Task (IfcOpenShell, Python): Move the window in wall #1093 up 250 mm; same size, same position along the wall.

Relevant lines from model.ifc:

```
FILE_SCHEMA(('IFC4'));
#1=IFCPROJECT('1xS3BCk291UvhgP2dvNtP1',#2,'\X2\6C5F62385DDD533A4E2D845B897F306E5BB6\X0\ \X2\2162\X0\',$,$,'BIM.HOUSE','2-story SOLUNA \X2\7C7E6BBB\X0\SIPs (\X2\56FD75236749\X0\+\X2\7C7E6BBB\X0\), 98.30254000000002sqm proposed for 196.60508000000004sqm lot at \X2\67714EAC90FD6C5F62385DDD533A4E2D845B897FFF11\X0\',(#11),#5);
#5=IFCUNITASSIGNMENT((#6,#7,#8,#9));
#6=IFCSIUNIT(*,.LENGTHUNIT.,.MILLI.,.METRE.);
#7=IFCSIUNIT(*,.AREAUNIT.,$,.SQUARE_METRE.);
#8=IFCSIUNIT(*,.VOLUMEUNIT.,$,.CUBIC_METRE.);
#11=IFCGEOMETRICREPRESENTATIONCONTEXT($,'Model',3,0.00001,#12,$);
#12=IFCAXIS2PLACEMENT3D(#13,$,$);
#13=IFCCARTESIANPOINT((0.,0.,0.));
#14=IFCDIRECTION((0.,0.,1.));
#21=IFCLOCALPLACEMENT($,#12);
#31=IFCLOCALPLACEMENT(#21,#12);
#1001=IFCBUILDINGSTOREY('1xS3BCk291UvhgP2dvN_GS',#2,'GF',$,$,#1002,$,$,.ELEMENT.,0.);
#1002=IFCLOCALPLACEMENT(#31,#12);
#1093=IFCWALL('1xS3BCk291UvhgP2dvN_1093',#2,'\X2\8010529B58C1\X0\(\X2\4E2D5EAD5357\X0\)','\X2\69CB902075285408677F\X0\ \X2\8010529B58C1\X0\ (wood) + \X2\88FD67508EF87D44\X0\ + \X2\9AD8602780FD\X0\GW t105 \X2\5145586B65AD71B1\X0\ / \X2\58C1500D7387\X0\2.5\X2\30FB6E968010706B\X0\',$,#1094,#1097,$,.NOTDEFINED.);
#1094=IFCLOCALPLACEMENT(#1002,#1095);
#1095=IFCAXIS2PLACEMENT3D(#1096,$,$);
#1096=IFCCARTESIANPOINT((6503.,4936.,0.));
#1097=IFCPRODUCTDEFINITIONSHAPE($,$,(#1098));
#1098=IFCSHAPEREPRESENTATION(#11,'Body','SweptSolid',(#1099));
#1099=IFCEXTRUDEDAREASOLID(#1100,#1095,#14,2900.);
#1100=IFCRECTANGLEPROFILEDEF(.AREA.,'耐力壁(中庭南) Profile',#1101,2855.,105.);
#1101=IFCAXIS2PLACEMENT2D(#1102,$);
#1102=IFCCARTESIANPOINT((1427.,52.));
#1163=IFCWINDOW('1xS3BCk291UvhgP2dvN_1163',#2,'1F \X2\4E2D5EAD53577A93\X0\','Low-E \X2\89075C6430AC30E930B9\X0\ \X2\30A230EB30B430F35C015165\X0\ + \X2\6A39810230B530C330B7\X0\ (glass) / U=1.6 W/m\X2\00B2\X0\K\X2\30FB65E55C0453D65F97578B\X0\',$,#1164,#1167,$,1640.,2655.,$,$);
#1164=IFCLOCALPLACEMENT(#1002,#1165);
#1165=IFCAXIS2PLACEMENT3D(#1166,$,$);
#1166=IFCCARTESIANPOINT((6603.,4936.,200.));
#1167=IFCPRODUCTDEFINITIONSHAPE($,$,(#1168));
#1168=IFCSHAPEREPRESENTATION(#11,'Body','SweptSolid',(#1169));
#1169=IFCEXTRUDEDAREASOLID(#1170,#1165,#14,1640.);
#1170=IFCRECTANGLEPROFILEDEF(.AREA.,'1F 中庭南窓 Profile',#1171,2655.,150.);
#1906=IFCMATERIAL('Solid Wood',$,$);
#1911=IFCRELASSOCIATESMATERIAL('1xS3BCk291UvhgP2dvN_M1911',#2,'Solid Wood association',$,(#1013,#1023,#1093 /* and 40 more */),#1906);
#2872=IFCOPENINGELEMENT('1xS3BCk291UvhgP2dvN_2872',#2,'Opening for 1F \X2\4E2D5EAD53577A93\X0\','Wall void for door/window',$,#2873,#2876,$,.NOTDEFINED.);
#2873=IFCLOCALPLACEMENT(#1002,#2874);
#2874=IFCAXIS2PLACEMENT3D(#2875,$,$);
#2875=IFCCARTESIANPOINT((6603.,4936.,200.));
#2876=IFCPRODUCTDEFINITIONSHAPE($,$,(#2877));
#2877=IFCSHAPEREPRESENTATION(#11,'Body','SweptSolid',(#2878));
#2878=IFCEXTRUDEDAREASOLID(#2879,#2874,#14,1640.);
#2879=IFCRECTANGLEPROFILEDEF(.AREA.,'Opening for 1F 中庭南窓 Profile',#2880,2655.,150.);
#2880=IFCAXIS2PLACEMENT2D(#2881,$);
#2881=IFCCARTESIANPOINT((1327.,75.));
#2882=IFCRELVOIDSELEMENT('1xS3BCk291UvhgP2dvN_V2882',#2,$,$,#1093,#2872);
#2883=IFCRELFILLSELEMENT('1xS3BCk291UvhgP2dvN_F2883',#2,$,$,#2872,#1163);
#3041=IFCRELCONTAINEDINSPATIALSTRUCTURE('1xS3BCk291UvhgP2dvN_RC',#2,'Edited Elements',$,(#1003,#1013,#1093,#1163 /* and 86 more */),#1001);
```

```python
import numpy as np
import ifcopenshell
import ifcopenshell.api.geometry
import ifcopenshell.util.placement
import ifcopenshell.util.unit

model = ifcopenshell.open("model.ifc")
unit_scale = ifcopenshell.util.unit.calculate_unit_scale(model)

window = model.by_id(1163)
opening = window.FillsVoids[0].RelatingOpeningElement
dz = 0.25 / unit_scale

shift = np.array([0.0, 0.0, dz])
# The window is not placed relative to its opening, so move both.
for product in (opening, window):
    matrix = ifcopenshell.util.placement.get_local_placement(product.ObjectPlacement)
    matrix[:3, 3] += shift
    ifcopenshell.api.geometry.edit_object_placement(model, product=product, matrix=matrix, is_si=False)

print(f"moved by {dz * unit_scale:+.3f} m")

model.write("model_edited.ifc")
```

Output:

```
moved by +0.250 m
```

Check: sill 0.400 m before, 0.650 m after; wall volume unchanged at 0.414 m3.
